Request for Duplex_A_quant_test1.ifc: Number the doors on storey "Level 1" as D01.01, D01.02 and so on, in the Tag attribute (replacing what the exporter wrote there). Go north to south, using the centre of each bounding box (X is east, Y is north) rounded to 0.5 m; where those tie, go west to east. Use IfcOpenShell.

First a look at what the model holds.

```python
import ifcopenshell
import ifcopenshell.util.element
import ifcopenshell.util.placement

model = ifcopenshell.open("Duplex_A_quant_test1.ifc")
print(model.schema)
storey = next(s for s in model.by_type("IfcBuildingStorey") if s.Name == "Level 1")
doors = [e for e in ifcopenshell.util.element.get_decomposition(storey) if e.is_a("IfcDoor")]
for e in sorted(doors, key=lambda e: e.id()):
    origin = ifcopenshell.util.placement.get_local_placement(e.ObjectPlacement)[:3, 3]
    print(e.id(), e.Tag, e.Name, origin.round(2) + 0.0, sep=" | ")
```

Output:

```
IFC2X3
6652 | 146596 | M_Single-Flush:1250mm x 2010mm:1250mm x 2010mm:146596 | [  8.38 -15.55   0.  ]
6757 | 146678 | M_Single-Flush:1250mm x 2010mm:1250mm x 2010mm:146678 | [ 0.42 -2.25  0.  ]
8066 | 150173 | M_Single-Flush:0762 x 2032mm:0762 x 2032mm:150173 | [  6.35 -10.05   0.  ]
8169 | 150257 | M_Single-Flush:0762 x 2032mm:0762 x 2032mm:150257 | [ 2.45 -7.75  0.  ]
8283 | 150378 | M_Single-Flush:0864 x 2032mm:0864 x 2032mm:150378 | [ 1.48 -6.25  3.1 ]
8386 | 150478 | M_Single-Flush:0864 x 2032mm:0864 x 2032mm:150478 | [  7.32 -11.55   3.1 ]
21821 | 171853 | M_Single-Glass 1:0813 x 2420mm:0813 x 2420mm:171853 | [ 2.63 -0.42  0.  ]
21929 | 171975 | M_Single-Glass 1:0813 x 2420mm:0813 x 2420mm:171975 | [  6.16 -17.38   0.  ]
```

```python
import ifcopenshell
import ifcopenshell.geom
import ifcopenshell.util.element
import ifcopenshell.util.shape

model = ifcopenshell.open("Duplex_A_quant_test1.ifc")
settings = ifcopenshell.geom.settings()
settings.set("use-world-coords", True)


def centre(element):
    shape = ifcopenshell.geom.create_shape(settings, element)
    return ifcopenshell.util.shape.get_bbox_centroid(shape.geometry)


storey = next(s for s in model.by_type("IfcBuildingStorey") if s.Name == "Level 1")
doors = [e for e in ifcopenshell.util.element.get_decomposition(storey) if e.is_a("IfcDoor")]

# Insertion points can sit at a corner or the storey origin, so sort by the geometry (in metres).
centres = {e: centre(e) for e in doors}
doors.sort(key=lambda e: (-round(centres[e][1] / 0.5), centres[e][0]))

for i, e in enumerate(doors, start=1):
    number = f"D01.{i:02d}"
    e.Tag = number
    print(e.id(), number)

model.write("Duplex_A_quant_test1_updated.ifc")
```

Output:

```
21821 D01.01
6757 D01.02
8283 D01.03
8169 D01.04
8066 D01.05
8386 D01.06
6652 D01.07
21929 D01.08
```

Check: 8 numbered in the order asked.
